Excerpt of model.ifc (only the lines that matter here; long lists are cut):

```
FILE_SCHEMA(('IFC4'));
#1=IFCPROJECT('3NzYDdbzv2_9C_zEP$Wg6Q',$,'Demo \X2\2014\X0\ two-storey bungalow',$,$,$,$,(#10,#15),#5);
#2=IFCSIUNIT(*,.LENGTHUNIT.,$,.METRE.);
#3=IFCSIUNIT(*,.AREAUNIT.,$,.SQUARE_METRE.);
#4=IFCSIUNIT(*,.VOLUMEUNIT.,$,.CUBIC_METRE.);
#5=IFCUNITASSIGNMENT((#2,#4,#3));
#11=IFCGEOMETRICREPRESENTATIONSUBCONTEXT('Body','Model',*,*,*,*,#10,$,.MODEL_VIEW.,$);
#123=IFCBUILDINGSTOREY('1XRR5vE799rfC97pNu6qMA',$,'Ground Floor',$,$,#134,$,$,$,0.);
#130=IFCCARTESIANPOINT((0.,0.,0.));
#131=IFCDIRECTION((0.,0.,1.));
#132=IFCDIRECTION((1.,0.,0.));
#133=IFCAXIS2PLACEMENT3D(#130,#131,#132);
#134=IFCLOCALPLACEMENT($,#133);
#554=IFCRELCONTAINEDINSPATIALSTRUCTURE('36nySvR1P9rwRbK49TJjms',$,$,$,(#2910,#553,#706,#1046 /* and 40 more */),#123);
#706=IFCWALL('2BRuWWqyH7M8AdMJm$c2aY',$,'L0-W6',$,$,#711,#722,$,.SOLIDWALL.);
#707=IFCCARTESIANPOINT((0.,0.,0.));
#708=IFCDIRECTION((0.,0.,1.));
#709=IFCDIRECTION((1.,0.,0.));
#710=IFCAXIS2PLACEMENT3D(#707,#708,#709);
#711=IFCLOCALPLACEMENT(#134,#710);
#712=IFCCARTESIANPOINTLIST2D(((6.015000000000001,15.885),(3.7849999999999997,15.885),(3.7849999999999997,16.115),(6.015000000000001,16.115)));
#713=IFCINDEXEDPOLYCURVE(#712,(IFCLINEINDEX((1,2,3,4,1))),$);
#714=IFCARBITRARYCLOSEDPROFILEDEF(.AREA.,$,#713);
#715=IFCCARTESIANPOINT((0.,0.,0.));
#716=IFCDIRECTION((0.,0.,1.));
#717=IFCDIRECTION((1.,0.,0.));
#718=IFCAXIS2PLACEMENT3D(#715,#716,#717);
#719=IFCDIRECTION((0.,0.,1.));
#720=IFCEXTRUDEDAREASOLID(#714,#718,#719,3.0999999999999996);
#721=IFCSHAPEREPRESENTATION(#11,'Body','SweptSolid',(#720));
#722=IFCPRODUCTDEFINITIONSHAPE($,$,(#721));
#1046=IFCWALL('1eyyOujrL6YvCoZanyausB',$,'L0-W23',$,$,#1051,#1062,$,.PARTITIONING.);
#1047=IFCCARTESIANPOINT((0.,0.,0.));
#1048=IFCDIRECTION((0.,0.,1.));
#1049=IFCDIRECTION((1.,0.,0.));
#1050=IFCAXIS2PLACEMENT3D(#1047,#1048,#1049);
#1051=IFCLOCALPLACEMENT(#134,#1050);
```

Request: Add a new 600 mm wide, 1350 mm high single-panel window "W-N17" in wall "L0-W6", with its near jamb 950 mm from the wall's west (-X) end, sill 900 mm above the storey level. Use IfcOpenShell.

```python
import numpy as np
import ifcopenshell
import ifcopenshell.api.feature
import ifcopenshell.api.geometry
import ifcopenshell.api.root
import ifcopenshell.api.spatial
import ifcopenshell.geom
import ifcopenshell.util.element
import ifcopenshell.util.placement
import ifcopenshell.util.representation
import ifcopenshell.util.shape
import ifcopenshell.util.unit

model = ifcopenshell.open("model.ifc")
unit_scale = ifcopenshell.util.unit.calculate_unit_scale(model)
settings = ifcopenshell.geom.settings()


def volume(element):
    """Net volume in cubic metres, openings subtracted."""
    shape = ifcopenshell.geom.create_shape(settings, element)
    return ifcopenshell.util.shape.get_volume(shape.geometry)


wall = model.by_guid("2BRuWWqyH7M8AdMJm$c2aY")
storey = ifcopenshell.util.element.get_container(wall, ifc_class="IfcBuildingStorey")
context = ifcopenshell.util.representation.get_context(model, "Model", "Body", "MODEL_VIEW")
before = volume(wall)

width, height, from_end, sill = 0.6, 1.35, 0.95, 0.9  # metres

# The wall runs along its own X axis, and the end named is its -X end.
wall_shape = ifcopenshell.geom.create_shape(settings, wall)
x, y, z = ifcopenshell.util.shape.get_vertices(wall_shape.geometry).T
start = x.min() + from_end
face, thickness = float(y.min()), float(y.max() - y.min())
wall_matrix = ifcopenshell.util.placement.get_local_placement(wall.ObjectPlacement)
level = ifcopenshell.util.placement.get_local_placement(storey.ObjectPlacement)[2, 3]


def in_wall(x, y):
    """Placement at x, y metres in the wall's axes, at sill height."""
    matrix = wall_matrix.copy()
    matrix[:, 3] = wall_matrix @ np.array([x / unit_scale, y / unit_scale, 0.0, 1.0])
    matrix[2, 3] = level + sill / unit_scale
    return matrix


# Opening: a box that overshoots both wall faces by 50 mm.
opening = ifcopenshell.api.root.create_entity(model, ifc_class="IfcOpeningElement", predefined_type="OPENING")
box = ifcopenshell.api.geometry.add_wall_representation(
    model, context=context, length=width, height=height, thickness=thickness + 0.1
)
ifcopenshell.api.geometry.assign_representation(model, product=opening, representation=box)
ifcopenshell.api.geometry.edit_object_placement(model, product=opening, matrix=in_wall(start, face - 0.05), is_si=False)
ifcopenshell.api.feature.add_feature(model, feature=opening, element=wall)

window = ifcopenshell.api.root.create_entity(model, ifc_class="IfcWindow", name="W-N17", predefined_type="WINDOW")
window.OverallWidth, window.OverallHeight = width / unit_scale, height / unit_scale
window.PartitioningType = "SINGLE_PANEL"
body = ifcopenshell.api.geometry.add_window_representation(
    model,
    context=context,
    overall_width=window.OverallWidth,
    overall_height=window.OverallHeight,
    partition_type="SINGLE_PANEL",
)
ifcopenshell.api.geometry.assign_representation(model, product=window, representation=body)
ifcopenshell.api.spatial.assign_container(model, products=[window], relating_structure=storey)
ifcopenshell.api.feature.add_filling(model, opening=opening, element=window)

# Centre the window in the wall's thickness.
ifcopenshell.api.geometry.edit_object_placement(model, product=window, matrix=in_wall(start, face), is_si=False)
window_shape = ifcopenshell.geom.create_shape(settings, window)
depth = ifcopenshell.util.shape.get_vertices(window_shape.geometry)[:, 1]
offset = face + thickness / 2 - (depth.min() + depth.max()) / 2
ifcopenshell.api.geometry.edit_object_placement(model, product=window, matrix=in_wall(start, offset), is_si=False)

after = volume(wall)

print(f"wall volume {before:.3f} -> {after:.3f} m3")

model.write("model_updated.ifc")
```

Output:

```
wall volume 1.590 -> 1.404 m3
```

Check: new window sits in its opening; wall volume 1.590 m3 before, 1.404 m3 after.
